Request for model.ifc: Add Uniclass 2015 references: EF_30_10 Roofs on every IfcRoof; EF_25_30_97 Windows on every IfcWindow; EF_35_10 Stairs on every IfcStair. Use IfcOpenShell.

First a look at what the model holds.

```python
import ifcopenshell

model = ifcopenshell.open("model.ifc")
print(model.schema)
print("classifications:", [c.Name for c in model.by_type("IfcClassification")])
for ifc_class in ("IfcDoor", "IfcRoof", "IfcStair", "IfcWall", "IfcWindow"):
    print(ifc_class, len(model.by_type(ifc_class)))
```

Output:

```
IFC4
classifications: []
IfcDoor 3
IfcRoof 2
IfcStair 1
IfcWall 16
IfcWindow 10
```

```python
import ifcopenshell
import ifcopenshell.api.classification

model = ifcopenshell.open("model.ifc")

system = ifcopenshell.api.classification.add_classification(model, classification="Uniclass 2015")

codes = {
    "IfcRoof": ("EF_30_10", "Roofs"),
    "IfcWindow": ("EF_25_30_97", "Windows"),
    "IfcStair": ("EF_35_10", "Stairs"),
}
for ifc_class, (code, name) in codes.items():
    products = model.by_type(ifc_class)
    ifcopenshell.api.classification.add_reference(
        model, products=products, classification=system, identification=code, name=name
    )
    print(code, len(products))

model.write("model_rev.ifc")
```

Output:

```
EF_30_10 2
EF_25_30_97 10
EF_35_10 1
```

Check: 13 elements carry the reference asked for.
